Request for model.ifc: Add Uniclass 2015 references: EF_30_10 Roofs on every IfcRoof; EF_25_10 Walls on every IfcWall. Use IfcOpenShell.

First a look at what the model holds.

```python
import ifcopenshell

model = ifcopenshell.open("model.ifc")
print(model.schema)
print("classifications:", [c.Name for c in model.by_type("IfcClassification")])
for ifc_class in ("IfcDoor", "IfcRoof", "IfcStair", "IfcWall", "IfcWindow"):
    print(ifc_class, len(model.by_type(ifc_class)))
```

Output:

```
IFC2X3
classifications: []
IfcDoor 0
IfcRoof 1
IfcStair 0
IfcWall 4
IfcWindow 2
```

```python
import ifcopenshell
import ifcopenshell.api.classification

model = ifcopenshell.open("model.ifc")

# IFC2X3 requires Source and Edition and has no link from the project to the system.
system = model.create_entity("IfcClassification", Source="NBS", Edition="2015", Name="Uniclass 2015")

codes = {
    "IfcRoof": ("EF_30_10", "Roofs"),
    "IfcWall": ("EF_25_10", "Walls"),
}
for ifc_class, (code, name) in codes.items():
    products = model.by_type(ifc_class)
    ifcopenshell.api.classification.add_reference(
        model, products=products, classification=system, identification=code, name=name
    )
    print(code, len(products))

model.write("model_rev.ifc")
```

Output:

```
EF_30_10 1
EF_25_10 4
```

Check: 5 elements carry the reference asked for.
